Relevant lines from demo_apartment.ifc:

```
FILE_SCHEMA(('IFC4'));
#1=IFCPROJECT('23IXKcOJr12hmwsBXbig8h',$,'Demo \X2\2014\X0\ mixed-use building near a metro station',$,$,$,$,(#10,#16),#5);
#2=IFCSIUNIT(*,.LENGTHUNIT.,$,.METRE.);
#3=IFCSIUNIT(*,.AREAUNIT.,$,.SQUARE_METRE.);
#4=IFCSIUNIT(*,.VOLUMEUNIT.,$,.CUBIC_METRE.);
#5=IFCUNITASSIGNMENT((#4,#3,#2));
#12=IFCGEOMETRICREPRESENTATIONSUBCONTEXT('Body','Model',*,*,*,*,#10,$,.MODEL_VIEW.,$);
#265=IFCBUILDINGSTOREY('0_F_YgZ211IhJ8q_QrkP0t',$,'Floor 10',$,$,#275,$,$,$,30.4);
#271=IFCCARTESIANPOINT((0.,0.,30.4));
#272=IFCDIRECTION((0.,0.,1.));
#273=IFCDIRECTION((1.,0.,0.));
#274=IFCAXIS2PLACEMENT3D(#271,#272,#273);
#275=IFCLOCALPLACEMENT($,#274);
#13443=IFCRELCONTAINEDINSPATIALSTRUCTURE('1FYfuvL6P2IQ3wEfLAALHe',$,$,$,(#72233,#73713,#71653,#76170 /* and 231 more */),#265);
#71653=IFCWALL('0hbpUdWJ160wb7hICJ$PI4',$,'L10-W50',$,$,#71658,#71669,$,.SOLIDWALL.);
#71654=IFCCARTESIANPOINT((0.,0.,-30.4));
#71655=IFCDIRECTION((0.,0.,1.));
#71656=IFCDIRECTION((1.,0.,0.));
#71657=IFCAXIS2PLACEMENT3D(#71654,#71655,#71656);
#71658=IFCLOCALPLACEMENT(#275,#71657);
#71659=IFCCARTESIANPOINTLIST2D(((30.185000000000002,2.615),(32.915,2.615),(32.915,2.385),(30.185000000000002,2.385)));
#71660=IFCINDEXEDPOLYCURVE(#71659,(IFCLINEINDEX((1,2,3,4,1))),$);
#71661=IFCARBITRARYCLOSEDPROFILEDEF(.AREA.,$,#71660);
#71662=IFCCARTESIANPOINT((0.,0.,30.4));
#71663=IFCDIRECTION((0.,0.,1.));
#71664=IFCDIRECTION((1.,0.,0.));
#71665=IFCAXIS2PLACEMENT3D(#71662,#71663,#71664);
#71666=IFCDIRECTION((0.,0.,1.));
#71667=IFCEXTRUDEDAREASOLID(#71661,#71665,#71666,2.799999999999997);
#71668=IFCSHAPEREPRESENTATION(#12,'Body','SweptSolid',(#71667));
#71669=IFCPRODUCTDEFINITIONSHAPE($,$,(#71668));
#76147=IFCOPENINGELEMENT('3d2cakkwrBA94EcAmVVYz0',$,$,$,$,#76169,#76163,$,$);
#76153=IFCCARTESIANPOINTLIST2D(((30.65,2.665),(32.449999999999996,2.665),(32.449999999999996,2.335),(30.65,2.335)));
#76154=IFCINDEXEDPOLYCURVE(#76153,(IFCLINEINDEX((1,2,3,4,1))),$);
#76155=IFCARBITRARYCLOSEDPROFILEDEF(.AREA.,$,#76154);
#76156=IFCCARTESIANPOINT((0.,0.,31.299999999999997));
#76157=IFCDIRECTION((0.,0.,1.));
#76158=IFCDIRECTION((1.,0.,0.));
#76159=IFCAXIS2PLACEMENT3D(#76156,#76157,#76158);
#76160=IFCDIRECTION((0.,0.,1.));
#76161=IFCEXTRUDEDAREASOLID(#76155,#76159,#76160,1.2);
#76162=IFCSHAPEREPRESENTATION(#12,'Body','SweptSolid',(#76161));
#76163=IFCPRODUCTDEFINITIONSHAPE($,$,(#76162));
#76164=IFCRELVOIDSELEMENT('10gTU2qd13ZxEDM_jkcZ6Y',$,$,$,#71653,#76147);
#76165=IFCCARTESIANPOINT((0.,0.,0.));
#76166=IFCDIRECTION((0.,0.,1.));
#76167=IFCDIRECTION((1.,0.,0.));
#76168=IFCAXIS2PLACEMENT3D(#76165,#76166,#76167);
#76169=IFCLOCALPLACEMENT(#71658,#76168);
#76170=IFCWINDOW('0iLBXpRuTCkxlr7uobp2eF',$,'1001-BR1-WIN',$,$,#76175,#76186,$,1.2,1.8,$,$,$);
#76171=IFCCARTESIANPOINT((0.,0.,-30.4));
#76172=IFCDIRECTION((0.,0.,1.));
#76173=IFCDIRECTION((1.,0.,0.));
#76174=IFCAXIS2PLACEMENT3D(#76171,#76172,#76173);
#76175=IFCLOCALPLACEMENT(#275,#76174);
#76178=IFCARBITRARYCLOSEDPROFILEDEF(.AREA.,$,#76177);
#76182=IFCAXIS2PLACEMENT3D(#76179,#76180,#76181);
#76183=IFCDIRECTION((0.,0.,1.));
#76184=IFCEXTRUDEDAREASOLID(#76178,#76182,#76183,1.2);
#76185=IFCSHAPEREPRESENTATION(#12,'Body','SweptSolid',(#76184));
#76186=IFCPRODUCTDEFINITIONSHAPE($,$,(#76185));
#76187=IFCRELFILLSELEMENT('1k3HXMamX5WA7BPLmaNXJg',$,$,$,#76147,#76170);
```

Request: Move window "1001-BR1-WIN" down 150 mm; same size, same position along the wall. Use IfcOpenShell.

```python
import numpy as np
import ifcopenshell
import ifcopenshell.api.geometry
import ifcopenshell.util.placement
import ifcopenshell.util.unit

model = ifcopenshell.open("demo_apartment.ifc")
unit_scale = ifcopenshell.util.unit.calculate_unit_scale(model)

window = model.by_guid("0iLBXpRuTCkxlr7uobp2eF")
opening = window.FillsVoids[0].RelatingOpeningElement
dz = -0.15 / unit_scale

shift = np.array([0.0, 0.0, dz])
# The window is not placed relative to its opening, so move both.
for product in (opening, window):
    matrix = ifcopenshell.util.placement.get_local_placement(product.ObjectPlacement)
    matrix[:3, 3] += shift
    ifcopenshell.api.geometry.edit_object_placement(model, product=product, matrix=matrix, is_si=False)

print(f"moved by {dz * unit_scale:+.3f} m")

model.write("demo_apartment-out.ifc")
```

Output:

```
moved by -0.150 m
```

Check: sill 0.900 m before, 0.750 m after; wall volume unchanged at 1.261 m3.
